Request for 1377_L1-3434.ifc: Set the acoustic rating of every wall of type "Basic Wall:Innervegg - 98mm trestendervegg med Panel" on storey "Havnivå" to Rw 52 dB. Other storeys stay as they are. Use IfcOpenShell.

First a look at what the model holds.

```python
import ifcopenshell
import ifcopenshell.util.element

model = ifcopenshell.open("1377_L1-3434.ifc")
print(model.schema)
storey = next(s for s in model.by_type("IfcBuildingStorey") if s.Name == "Havnivå")
walls = [e for e in ifcopenshell.util.element.get_decomposition(storey) if e.is_a("IfcWall")]
seen = {}
for e in walls:
    element_type = ifcopenshell.util.element.get_type(e)
    key = (element_type.Name if element_type != e and element_type else None, ifcopenshell.util.element.get_pset(e, "Pset_WallCommon", "AcousticRating"))
    seen[key] = seen.get(key, 0) + 1
for (name, value), count in sorted(seen.items(), key=str):
    print(count, "x", name, "|", value)
```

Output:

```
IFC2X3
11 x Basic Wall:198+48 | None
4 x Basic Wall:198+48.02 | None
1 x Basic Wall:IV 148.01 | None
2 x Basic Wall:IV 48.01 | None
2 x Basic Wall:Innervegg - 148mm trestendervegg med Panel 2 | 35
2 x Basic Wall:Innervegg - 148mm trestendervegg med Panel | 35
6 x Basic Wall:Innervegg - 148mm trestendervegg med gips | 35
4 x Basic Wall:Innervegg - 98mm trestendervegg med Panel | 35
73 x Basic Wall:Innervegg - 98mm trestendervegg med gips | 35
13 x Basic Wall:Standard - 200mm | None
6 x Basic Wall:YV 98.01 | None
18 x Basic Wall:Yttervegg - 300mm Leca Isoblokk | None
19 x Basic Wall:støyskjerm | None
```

```python
import ifcopenshell
import ifcopenshell.api.pset
import ifcopenshell.util.element

model = ifcopenshell.open("1377_L1-3434.ifc")

storey = next(s for s in model.by_type("IfcBuildingStorey") if s.Name == "Havnivå")
walls = [e for e in ifcopenshell.util.element.get_decomposition(storey) if e.is_a("IfcWall")]

count = 0
for e in walls:
    element_type = ifcopenshell.util.element.get_type(e)
    if element_type in (None, e) or element_type.Name != "Basic Wall:Innervegg - 98mm trestendervegg med Panel":
        continue
    # add_pset returns the element's existing set when there is one.
    pset = ifcopenshell.api.pset.add_pset(model, product=e, name="Pset_WallCommon")
    ifcopenshell.api.pset.edit_pset(model, pset=pset, properties={"AcousticRating": "Rw 52 dB"})
    count += 1

print(count, "walls updated")

model.write("1377_L1-3434_edited.ifc")
```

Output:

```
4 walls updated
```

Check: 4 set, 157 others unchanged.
